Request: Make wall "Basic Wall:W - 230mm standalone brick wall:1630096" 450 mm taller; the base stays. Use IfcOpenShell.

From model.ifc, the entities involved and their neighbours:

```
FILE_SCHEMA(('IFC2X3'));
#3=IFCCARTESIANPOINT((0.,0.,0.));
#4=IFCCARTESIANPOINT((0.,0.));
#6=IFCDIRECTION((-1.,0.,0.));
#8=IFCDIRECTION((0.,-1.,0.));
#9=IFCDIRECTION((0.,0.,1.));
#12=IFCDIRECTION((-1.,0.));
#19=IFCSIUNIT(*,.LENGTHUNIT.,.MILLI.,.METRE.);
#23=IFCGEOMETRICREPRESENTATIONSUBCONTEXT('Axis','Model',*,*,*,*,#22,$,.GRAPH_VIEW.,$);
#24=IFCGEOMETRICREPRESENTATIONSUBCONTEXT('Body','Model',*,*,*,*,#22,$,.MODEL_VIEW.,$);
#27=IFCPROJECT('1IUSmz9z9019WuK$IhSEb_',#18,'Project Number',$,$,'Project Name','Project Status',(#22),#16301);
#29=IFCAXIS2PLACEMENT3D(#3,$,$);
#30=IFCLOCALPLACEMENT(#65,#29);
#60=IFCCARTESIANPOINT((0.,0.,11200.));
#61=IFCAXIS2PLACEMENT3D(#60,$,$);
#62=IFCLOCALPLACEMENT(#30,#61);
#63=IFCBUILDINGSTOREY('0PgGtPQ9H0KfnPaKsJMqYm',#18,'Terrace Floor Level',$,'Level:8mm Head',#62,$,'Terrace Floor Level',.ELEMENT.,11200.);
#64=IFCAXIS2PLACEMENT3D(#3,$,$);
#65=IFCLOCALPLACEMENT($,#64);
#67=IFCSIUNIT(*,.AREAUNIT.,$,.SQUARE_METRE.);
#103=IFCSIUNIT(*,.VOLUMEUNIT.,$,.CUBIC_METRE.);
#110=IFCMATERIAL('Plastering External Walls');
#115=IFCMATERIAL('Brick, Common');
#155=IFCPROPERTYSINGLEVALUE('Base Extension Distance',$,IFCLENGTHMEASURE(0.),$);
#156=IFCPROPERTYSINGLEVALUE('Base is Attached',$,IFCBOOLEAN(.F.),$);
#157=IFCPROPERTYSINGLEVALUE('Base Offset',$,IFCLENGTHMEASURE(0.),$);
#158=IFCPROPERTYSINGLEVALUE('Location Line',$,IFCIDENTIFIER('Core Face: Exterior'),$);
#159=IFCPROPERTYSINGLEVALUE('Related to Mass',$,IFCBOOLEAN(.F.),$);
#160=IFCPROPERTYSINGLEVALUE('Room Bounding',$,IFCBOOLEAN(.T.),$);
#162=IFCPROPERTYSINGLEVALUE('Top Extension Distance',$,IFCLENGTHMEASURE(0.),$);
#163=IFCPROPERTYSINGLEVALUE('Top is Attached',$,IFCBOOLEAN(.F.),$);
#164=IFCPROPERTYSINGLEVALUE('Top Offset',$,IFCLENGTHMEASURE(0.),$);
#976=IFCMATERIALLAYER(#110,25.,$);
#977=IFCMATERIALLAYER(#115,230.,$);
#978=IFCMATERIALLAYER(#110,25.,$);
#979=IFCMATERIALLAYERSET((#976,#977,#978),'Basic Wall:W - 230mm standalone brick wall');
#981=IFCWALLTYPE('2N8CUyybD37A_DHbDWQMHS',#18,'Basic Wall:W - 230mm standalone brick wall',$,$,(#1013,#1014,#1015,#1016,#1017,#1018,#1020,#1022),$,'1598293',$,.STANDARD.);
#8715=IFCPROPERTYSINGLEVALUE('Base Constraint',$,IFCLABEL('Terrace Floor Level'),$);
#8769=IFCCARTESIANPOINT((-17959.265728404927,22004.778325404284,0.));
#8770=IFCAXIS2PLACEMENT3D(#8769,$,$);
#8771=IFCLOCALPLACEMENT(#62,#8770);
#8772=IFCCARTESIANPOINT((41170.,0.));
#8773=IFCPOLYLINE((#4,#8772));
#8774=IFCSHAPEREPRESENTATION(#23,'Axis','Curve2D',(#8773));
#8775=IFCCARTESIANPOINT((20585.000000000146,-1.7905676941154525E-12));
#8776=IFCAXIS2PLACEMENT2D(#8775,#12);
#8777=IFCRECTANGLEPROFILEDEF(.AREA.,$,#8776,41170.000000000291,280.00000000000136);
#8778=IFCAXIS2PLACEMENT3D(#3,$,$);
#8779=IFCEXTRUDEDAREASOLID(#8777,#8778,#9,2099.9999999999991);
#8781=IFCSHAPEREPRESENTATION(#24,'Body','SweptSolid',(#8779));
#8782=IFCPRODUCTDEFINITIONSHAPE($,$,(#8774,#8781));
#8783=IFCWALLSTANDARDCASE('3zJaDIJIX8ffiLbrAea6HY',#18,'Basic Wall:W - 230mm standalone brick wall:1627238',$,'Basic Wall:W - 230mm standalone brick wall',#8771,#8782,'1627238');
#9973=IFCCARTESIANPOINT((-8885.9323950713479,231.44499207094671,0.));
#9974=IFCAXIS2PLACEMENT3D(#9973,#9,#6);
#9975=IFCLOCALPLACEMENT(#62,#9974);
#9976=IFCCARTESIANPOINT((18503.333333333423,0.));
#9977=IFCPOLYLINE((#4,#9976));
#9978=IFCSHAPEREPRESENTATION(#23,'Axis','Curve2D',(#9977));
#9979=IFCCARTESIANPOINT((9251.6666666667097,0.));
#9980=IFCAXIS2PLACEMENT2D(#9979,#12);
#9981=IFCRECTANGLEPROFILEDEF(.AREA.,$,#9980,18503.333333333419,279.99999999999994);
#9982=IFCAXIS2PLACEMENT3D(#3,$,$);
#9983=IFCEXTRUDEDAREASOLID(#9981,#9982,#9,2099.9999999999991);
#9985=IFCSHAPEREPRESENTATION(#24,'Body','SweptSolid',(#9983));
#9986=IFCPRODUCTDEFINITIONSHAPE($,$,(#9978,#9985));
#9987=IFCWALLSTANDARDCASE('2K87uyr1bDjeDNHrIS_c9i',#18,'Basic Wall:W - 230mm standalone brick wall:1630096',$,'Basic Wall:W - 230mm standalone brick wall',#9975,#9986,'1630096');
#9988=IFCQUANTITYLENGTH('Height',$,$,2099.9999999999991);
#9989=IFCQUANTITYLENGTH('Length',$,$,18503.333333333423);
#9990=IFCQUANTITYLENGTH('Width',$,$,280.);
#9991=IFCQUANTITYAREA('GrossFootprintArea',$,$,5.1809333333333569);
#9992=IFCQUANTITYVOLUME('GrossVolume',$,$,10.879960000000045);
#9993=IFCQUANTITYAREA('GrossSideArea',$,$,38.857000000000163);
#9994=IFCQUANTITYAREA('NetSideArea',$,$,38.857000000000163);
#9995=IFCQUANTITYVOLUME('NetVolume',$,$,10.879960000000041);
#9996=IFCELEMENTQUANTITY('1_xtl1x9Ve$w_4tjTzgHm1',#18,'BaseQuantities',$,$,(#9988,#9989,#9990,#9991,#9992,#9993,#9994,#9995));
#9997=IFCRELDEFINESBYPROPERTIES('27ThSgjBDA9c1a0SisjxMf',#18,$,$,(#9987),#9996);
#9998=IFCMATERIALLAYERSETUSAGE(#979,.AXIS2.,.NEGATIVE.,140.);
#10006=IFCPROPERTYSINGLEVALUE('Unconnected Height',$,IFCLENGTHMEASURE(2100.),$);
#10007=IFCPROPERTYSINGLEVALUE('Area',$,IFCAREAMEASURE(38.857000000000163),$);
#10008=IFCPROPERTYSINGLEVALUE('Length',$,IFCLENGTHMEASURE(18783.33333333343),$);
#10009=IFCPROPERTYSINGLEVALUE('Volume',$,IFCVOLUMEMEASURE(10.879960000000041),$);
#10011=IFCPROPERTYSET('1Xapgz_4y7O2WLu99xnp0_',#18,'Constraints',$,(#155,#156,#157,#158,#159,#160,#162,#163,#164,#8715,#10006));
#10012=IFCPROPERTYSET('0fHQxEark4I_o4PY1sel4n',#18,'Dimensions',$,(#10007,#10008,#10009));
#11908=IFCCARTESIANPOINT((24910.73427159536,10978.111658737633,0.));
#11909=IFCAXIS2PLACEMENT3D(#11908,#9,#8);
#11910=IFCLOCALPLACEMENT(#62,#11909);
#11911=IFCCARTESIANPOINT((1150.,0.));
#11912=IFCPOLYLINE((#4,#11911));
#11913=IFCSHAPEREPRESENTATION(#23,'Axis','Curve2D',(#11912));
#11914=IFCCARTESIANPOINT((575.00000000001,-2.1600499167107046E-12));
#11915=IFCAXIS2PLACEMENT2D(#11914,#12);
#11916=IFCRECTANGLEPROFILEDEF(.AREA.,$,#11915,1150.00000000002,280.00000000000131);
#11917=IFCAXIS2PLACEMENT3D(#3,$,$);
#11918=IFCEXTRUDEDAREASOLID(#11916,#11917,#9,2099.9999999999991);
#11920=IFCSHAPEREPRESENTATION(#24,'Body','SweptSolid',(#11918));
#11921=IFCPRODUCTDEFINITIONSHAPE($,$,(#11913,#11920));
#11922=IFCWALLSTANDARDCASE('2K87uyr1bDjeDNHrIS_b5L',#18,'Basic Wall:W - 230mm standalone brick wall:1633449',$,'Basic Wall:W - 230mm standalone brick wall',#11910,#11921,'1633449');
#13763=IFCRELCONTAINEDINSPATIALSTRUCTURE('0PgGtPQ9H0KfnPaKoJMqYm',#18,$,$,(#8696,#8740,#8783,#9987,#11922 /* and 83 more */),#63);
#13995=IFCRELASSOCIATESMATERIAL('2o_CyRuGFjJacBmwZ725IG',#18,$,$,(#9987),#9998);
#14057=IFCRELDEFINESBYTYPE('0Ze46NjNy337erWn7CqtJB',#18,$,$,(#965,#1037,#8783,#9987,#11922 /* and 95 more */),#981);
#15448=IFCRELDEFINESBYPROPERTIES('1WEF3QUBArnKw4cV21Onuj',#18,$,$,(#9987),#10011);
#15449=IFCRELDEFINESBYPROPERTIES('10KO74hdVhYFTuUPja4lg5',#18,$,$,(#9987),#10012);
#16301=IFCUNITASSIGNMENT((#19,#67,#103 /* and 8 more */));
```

```python
import ifcopenshell
import ifcopenshell.api.pset
import ifcopenshell.geom
import ifcopenshell.util.element
import ifcopenshell.util.representation
import ifcopenshell.util.shape
import ifcopenshell.util.unit

model = ifcopenshell.open("model.ifc")
unit_scale = ifcopenshell.util.unit.calculate_unit_scale(model)
area_scale = ifcopenshell.util.unit.calculate_unit_scale(model, "AREAUNIT")
volume_scale = ifcopenshell.util.unit.calculate_unit_scale(model, "VOLUMEUNIT")
settings = ifcopenshell.geom.settings()


def volume(element):
    """Net volume in cubic metres, openings subtracted."""
    shape = ifcopenshell.geom.create_shape(settings, element)
    return ifcopenshell.util.shape.get_volume(shape.geometry)


wall = model.by_guid("2K87uyr1bDjeDNHrIS_c9i")
before = volume(wall)

body = ifcopenshell.util.representation.get_representation(wall, "Model", "Body")
solid = body.Items[0]
old_height = solid.Depth
solid.Depth += 0.45 / unit_scale
after = volume(wall)
thickness = 0.28  # wall thickness in metres

# Update the stored height, areas and volumes.
qto = model.by_id(ifcopenshell.util.element.get_pset(wall, "BaseQuantities", should_inherit=False)["id"])
ifcopenshell.api.pset.edit_qto(model, qto=qto, properties={
    "Height": solid.Depth,
    "GrossVolume": ifcopenshell.util.element.get_pset(wall, "BaseQuantities", "GrossVolume") * solid.Depth / old_height,
    "GrossSideArea": ifcopenshell.util.element.get_pset(wall, "BaseQuantities", "GrossSideArea") * solid.Depth / old_height,
    "NetSideArea": after / thickness / area_scale,
    "NetVolume": after / volume_scale,
})
pset = model.by_id(ifcopenshell.util.element.get_pset(wall, "Constraints", should_inherit=False)["id"])
ifcopenshell.api.pset.edit_pset(model, pset=pset, properties={
    "Unconnected Height": model.create_entity("IfcLengthMeasure", solid.Depth),
})
pset = model.by_id(ifcopenshell.util.element.get_pset(wall, "Dimensions", should_inherit=False)["id"])
ifcopenshell.api.pset.edit_pset(model, pset=pset, properties={
    "Area": model.create_entity("IfcAreaMeasure", after / thickness / area_scale),
    "Volume": model.create_entity("IfcVolumeMeasure", after / volume_scale),
})

print(f"height {old_height:g} -> {solid.Depth:g}, volume {before:.3f} -> {after:.3f} m3")

model.write("model_edited.ifc")
```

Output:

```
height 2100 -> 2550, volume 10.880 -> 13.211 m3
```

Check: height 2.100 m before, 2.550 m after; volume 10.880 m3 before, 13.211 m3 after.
